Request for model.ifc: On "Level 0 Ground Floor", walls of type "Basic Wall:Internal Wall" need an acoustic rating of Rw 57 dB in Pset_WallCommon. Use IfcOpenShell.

First a look at what the model holds.

```python
import ifcopenshell
import ifcopenshell.util.element

model = ifcopenshell.open("model.ifc")
print(model.schema)
storey = next(s for s in model.by_type("IfcBuildingStorey") if s.Name == "Level 0 Ground Floor")
walls = [e for e in ifcopenshell.util.element.get_decomposition(storey) if e.is_a("IfcWall")]
seen = {}
for e in walls:
    element_type = ifcopenshell.util.element.get_type(e)
    key = (element_type.Name if element_type != e and element_type else None, ifcopenshell.util.element.get_pset(e, "Pset_WallCommon", "AcousticRating"))
    seen[key] = seen.get(key, 0) + 1
for (name, value), count in sorted(seen.items(), key=str):
    print(count, "x", name, "|", value)
```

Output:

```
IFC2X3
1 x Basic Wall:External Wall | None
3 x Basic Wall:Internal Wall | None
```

```python
import ifcopenshell
import ifcopenshell.api.pset
import ifcopenshell.util.element

model = ifcopenshell.open("model.ifc")

storey = next(s for s in model.by_type("IfcBuildingStorey") if s.Name == "Level 0 Ground Floor")
walls = [e for e in ifcopenshell.util.element.get_decomposition(storey) if e.is_a("IfcWall")]

count = 0
for e in walls:
    element_type = ifcopenshell.util.element.get_type(e)
    if element_type in (None, e) or element_type.Name != "Basic Wall:Internal Wall":
        continue
    # add_pset returns the element's existing set when there is one.
    pset = ifcopenshell.api.pset.add_pset(model, product=e, name="Pset_WallCommon")
    ifcopenshell.api.pset.edit_pset(model, pset=pset, properties={"AcousticRating": "Rw 57 dB"})
    count += 1

print(count, "walls updated")

model.write("model_updated.ifc")
```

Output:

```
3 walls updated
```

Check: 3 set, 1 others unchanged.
